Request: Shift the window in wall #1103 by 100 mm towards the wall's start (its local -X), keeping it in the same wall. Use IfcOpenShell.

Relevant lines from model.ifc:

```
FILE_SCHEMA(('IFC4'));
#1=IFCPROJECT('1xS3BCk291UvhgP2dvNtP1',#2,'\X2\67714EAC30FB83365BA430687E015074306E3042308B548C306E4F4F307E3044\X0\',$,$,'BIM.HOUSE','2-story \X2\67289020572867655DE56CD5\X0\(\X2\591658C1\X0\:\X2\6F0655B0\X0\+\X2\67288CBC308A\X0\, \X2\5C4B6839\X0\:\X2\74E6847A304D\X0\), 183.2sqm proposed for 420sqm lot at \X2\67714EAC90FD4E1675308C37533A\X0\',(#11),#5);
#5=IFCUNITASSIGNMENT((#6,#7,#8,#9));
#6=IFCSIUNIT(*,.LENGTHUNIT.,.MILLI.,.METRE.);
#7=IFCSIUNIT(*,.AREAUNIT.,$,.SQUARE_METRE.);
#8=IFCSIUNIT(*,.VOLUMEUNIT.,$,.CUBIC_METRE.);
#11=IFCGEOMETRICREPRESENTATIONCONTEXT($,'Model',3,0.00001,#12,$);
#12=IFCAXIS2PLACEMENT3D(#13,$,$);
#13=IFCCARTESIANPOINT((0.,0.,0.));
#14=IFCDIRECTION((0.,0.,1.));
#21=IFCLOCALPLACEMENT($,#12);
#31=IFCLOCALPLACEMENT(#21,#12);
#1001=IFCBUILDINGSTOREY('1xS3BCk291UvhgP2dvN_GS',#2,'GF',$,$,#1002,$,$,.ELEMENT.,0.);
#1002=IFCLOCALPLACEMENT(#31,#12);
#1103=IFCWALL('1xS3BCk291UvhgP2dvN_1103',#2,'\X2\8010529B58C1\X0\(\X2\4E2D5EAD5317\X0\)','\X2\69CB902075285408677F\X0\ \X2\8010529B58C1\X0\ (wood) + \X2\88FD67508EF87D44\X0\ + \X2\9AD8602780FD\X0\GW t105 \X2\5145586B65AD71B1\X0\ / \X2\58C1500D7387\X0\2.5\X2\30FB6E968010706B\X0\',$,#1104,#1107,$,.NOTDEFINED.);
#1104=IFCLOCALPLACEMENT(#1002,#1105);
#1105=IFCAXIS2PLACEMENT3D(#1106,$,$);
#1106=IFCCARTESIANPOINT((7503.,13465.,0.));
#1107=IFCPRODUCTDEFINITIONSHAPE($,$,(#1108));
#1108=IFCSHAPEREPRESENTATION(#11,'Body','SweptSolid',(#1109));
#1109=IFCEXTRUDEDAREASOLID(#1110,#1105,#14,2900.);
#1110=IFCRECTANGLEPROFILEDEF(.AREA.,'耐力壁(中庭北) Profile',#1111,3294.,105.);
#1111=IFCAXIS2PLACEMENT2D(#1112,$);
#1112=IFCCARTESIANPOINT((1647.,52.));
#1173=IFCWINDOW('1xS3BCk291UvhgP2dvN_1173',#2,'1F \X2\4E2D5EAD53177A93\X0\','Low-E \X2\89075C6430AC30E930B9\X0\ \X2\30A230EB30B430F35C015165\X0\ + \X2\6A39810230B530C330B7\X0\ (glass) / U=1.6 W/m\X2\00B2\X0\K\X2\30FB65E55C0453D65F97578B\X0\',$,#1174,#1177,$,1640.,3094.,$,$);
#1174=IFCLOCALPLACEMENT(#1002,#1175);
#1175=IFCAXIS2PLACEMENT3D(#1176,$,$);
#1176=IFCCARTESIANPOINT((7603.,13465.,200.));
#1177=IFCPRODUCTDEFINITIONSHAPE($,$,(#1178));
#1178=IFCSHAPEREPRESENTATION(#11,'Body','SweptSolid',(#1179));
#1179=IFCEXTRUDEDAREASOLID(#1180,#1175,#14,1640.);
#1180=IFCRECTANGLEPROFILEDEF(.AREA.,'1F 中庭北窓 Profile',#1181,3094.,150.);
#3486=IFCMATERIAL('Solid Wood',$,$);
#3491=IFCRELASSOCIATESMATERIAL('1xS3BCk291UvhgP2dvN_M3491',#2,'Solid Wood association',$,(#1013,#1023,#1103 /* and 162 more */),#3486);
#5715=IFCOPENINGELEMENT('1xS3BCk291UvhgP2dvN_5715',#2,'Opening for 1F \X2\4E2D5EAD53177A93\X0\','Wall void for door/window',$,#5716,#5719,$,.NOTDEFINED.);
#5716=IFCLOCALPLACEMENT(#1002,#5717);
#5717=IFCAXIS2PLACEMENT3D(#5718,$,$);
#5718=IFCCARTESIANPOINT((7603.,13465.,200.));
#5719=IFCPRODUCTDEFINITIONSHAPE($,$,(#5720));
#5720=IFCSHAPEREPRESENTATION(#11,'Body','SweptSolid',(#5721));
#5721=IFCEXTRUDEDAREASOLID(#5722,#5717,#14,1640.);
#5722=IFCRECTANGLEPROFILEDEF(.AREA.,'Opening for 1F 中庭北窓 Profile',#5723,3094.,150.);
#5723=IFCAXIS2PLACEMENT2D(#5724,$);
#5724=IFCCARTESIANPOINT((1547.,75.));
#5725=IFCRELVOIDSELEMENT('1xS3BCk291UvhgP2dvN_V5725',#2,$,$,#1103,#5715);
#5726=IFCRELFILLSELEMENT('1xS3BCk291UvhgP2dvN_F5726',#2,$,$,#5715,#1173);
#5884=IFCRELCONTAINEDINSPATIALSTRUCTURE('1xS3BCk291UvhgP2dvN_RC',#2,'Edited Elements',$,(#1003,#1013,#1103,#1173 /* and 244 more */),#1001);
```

```python
import ifcopenshell
import ifcopenshell.api.geometry
import ifcopenshell.util.placement
import ifcopenshell.util.unit

model = ifcopenshell.open("model.ifc")
unit_scale = ifcopenshell.util.unit.calculate_unit_scale(model)

window = model.by_id(1173)
opening = window.FillsVoids[0].RelatingOpeningElement
wall = opening.VoidsElements[0].RelatingBuildingElement

wall_matrix = ifcopenshell.util.placement.get_local_placement(wall.ObjectPlacement)
shift = wall_matrix[:3, 0] * -0.1 / unit_scale
before = ifcopenshell.util.placement.get_local_placement(window.ObjectPlacement)[:3, 3].copy()

# The window is not placed relative to its opening, so move both.
for product in (opening, window):
    matrix = ifcopenshell.util.placement.get_local_placement(product.ObjectPlacement)
    matrix[:3, 3] += shift
    ifcopenshell.api.geometry.edit_object_placement(model, product=product, matrix=matrix, is_si=False)

after = ifcopenshell.util.placement.get_local_placement(window.ObjectPlacement)[:3, 3]
print("window moved by", (after - before).round(3) + 0.0)

model.write("model_updated.ifc")
```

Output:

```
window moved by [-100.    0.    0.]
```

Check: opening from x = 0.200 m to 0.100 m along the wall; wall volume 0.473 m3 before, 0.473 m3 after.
